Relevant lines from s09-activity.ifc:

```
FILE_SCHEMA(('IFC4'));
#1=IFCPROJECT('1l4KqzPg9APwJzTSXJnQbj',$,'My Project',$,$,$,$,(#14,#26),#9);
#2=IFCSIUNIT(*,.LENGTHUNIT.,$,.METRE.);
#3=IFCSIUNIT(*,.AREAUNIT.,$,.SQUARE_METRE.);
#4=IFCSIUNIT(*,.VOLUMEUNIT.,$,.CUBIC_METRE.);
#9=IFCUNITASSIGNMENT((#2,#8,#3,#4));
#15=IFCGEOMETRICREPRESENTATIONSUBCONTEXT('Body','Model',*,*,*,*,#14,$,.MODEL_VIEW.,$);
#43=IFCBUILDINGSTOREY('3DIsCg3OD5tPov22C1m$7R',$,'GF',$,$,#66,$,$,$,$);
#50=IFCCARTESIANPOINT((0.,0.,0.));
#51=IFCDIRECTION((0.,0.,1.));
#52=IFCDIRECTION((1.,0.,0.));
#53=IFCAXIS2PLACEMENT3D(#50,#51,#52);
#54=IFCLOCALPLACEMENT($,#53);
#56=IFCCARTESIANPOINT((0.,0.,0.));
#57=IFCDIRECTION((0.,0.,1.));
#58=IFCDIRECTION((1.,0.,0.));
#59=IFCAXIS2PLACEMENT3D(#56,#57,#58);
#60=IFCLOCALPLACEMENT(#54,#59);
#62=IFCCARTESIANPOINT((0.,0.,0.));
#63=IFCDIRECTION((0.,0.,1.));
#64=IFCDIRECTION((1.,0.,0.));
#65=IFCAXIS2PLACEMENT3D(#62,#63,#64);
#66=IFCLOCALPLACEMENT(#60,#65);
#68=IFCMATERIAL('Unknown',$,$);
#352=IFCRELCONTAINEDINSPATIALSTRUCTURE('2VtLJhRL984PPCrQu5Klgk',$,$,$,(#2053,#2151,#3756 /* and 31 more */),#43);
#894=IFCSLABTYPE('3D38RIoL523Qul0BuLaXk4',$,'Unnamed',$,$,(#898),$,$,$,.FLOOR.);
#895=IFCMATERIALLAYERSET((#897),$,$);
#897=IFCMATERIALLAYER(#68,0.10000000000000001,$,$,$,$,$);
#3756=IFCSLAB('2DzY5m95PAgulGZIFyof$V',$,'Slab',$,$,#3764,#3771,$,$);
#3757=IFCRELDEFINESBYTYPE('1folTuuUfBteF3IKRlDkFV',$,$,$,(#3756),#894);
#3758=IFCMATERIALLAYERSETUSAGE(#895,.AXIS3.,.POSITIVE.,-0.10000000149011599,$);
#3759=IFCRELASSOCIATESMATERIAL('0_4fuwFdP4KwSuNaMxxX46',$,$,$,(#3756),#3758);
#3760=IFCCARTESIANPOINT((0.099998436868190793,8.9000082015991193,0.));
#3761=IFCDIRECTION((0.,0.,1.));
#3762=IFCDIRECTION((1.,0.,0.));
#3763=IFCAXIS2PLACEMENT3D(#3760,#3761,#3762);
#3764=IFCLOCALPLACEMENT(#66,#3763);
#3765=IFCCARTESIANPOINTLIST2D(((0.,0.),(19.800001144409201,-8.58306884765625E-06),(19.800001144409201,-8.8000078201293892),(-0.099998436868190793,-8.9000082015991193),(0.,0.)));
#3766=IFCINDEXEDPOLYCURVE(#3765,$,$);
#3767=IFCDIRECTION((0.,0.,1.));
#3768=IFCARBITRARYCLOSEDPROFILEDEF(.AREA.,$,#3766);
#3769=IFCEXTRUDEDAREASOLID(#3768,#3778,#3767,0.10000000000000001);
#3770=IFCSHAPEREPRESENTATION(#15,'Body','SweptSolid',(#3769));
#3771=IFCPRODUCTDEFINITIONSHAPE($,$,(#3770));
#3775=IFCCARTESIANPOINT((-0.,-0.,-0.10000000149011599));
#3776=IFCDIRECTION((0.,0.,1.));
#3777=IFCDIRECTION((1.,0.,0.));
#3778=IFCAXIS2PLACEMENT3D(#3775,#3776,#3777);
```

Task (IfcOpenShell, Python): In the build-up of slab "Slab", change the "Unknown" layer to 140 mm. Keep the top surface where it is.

```python
import ifcopenshell
import ifcopenshell.util.element
import ifcopenshell.util.representation
import ifcopenshell.util.unit

model = ifcopenshell.open("s09-activity.ifc")
unit_scale = ifcopenshell.util.unit.calculate_unit_scale(model)

layer_set = model.by_id(895)
layer = next(l for l in layer_set.MaterialLayers if l.Material and l.Material.Name == "Unknown")
change = 0.14 / unit_scale - layer.LayerThickness
layer.LayerThickness += change

# Geometry does not follow the layer set by itself.
slabs = [e for e in ifcopenshell.util.element.get_elements_by_material(model, layer_set) if e.is_a("IfcSlab")]
for slab in sorted(slabs, key=lambda e: e.id()):
    body = ifcopenshell.util.representation.get_representation(slab, "Model", "Body")
    solid = body.Items[0]
    old_depth = solid.Depth
    solid.Depth += change
    # Extruded upwards: lower the start of the extrusion so the top stays.
    x, y, z = solid.Position.Location.Coordinates
    solid.Position.Location = model.createIfcCartesianPoint((x, y, z - change))
    print(slab.id(), f"{old_depth:g} -> {solid.Depth:g}")

# The layers are counted up from the underside, which has moved.
for usage in {ifcopenshell.util.element.get_material(slab) for slab in slabs}:
    usage.OffsetFromReferenceLine -= change

model.write("s09-activity_v2.ifc")
```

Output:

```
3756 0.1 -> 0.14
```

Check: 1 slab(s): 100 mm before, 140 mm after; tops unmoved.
